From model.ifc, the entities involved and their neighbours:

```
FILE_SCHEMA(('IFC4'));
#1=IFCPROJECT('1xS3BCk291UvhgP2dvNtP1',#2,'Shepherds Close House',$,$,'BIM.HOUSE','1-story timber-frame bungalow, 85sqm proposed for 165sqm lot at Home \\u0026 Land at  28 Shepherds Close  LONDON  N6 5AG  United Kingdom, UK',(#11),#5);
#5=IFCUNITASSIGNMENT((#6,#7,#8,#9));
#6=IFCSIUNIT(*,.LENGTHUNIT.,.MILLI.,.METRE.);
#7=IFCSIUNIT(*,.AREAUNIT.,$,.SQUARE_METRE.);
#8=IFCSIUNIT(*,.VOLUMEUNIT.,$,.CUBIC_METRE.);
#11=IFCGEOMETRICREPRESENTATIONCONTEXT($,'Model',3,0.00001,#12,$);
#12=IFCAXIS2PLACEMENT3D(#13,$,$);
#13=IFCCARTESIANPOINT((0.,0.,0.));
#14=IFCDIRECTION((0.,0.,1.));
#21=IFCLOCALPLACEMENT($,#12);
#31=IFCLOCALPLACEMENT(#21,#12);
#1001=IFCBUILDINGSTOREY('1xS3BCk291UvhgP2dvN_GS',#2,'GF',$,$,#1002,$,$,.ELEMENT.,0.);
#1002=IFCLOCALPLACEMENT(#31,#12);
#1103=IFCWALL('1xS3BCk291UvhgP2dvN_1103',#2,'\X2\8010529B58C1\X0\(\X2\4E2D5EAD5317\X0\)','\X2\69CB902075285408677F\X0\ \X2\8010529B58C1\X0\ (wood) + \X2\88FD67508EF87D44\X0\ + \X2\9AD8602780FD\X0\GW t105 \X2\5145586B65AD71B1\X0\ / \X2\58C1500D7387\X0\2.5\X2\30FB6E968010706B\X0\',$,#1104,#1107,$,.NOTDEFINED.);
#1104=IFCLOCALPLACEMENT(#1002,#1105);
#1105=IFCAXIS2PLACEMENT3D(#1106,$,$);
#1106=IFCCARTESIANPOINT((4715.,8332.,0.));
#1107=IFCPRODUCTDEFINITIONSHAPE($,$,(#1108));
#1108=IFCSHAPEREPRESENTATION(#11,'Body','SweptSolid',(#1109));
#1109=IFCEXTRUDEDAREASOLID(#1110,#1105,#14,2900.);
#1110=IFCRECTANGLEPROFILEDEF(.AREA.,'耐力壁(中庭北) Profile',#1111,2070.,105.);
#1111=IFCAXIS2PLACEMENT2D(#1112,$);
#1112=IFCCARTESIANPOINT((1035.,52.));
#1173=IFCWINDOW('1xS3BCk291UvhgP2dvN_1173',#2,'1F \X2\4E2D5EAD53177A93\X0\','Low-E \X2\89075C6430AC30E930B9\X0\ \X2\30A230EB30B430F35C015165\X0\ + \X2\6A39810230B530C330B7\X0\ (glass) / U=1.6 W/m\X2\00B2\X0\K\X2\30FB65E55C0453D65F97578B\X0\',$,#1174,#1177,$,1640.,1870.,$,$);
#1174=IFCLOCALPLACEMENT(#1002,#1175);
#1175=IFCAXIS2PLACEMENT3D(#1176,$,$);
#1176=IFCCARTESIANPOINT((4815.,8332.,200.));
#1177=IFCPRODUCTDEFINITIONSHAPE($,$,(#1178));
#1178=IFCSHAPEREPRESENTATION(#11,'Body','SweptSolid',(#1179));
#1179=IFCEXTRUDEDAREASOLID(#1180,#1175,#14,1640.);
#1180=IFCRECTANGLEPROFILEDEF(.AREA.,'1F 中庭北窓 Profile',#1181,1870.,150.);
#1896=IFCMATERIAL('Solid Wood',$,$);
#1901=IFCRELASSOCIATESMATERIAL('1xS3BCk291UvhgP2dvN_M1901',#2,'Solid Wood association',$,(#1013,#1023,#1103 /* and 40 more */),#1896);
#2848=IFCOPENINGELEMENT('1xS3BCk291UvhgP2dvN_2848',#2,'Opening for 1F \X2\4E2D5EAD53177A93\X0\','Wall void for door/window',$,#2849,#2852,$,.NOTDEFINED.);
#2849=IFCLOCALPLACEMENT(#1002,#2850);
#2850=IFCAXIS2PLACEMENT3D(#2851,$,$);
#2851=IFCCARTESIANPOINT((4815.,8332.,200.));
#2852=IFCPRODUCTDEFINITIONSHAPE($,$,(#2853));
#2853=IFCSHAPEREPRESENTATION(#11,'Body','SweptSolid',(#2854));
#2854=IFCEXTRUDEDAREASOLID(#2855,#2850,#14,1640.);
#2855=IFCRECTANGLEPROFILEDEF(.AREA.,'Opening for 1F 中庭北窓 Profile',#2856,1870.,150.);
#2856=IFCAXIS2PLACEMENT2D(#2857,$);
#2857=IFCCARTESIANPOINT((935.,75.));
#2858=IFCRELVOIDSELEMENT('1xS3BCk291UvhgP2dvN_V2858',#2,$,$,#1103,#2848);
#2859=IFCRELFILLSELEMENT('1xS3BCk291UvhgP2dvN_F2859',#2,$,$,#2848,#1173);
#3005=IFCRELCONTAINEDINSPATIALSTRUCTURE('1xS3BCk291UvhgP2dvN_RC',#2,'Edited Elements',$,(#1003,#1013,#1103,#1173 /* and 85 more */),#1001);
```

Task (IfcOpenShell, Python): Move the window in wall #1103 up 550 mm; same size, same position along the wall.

```python
import numpy as np
import ifcopenshell
import ifcopenshell.api.geometry
import ifcopenshell.util.placement
import ifcopenshell.util.unit

model = ifcopenshell.open("model.ifc")
unit_scale = ifcopenshell.util.unit.calculate_unit_scale(model)

window = model.by_guid("1xS3BCk291UvhgP2dvN_1173")
opening = window.FillsVoids[0].RelatingOpeningElement
dz = 0.55 / unit_scale

shift = np.array([0.0, 0.0, dz])
# The window is not placed relative to its opening, so move both.
for product in (opening, window):
    matrix = ifcopenshell.util.placement.get_local_placement(product.ObjectPlacement)
    matrix[:3, 3] += shift
    ifcopenshell.api.geometry.edit_object_placement(model, product=product, matrix=matrix, is_si=False)

print(f"moved by {dz * unit_scale:+.3f} m")

model.write("model-out.ifc")
```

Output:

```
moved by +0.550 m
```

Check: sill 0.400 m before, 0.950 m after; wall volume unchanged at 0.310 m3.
